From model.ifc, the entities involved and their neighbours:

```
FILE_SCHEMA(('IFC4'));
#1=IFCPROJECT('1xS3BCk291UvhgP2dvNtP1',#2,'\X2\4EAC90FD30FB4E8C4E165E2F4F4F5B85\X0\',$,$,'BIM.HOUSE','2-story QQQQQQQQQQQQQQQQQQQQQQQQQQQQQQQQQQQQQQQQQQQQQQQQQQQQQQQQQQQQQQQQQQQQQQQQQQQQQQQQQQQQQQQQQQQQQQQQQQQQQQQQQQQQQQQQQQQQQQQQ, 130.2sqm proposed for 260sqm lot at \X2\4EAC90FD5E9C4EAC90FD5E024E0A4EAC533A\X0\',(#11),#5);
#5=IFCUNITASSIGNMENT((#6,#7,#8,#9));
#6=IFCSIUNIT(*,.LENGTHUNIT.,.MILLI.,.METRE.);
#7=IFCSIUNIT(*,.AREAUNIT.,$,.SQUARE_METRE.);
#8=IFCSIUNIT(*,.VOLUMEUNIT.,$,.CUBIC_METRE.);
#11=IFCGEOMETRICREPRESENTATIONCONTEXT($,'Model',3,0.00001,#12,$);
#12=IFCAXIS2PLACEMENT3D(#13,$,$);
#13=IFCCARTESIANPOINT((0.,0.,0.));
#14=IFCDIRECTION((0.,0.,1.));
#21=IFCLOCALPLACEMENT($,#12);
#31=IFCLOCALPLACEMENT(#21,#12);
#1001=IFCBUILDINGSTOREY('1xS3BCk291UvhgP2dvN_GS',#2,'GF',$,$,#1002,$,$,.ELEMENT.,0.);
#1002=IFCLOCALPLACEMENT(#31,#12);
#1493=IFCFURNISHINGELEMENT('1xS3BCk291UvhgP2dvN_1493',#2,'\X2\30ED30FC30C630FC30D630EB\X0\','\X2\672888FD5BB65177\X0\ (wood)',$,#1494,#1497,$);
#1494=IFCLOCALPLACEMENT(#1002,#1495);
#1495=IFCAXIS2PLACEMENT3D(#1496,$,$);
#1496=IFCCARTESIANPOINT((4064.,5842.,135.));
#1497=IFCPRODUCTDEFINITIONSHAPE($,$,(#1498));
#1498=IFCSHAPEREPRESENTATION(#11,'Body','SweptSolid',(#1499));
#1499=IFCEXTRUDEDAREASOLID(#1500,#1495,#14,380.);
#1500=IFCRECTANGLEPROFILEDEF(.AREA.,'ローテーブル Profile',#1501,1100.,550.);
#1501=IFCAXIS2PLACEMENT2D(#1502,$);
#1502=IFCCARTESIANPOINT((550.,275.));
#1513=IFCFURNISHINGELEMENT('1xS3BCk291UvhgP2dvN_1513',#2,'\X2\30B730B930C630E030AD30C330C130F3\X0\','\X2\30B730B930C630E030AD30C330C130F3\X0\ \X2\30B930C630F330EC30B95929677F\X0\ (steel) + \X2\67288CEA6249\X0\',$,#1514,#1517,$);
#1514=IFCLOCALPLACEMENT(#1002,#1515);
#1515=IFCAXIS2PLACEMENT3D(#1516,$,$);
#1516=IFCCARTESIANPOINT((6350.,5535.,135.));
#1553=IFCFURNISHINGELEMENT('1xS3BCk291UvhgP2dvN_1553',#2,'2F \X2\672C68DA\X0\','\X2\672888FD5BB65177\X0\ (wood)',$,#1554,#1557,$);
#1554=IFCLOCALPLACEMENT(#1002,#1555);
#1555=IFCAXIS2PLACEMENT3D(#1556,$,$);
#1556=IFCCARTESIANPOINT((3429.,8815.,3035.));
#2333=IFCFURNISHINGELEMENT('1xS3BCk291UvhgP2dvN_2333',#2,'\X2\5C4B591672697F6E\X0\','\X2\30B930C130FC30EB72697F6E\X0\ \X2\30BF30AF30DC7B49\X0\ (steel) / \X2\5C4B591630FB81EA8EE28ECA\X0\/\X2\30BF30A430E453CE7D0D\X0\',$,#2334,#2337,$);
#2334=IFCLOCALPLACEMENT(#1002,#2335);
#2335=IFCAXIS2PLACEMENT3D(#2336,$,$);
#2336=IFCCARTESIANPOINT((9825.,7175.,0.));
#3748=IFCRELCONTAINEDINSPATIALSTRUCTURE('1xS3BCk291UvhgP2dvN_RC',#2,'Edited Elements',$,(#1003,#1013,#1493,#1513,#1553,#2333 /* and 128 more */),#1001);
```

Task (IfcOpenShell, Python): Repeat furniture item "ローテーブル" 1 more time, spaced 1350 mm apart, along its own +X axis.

```python
import ifcopenshell
import ifcopenshell.api.geometry
import ifcopenshell.api.root
import ifcopenshell.util.element
import ifcopenshell.util.placement
import ifcopenshell.util.unit

model = ifcopenshell.open("model.ifc")
unit_scale = ifcopenshell.util.unit.calculate_unit_scale(model)


def reuse_history(source, copy):
    """copy_class also copies each property set's owner history, people and application; keep the originals."""
    for rel in copy.IsDefinedBy:
        if rel.is_a("IfcRelDefinesByProperties") and (history := rel.RelatingPropertyDefinition.OwnerHistory):
            rel.RelatingPropertyDefinition.OwnerHistory = source.OwnerHistory
            ifcopenshell.util.element.remove_deep2(model, history)


source = model.by_guid("1xS3BCk291UvhgP2dvN_1493")
base = ifcopenshell.util.placement.get_local_placement(source.ObjectPlacement)
step = base[:3, 0] * 1.35 / unit_scale

for i in range(1, 2):
    copy = ifcopenshell.api.root.copy_class(model, product=source)
    copy.Representation = ifcopenshell.util.element.copy_deep(
        model, source.Representation, exclude=["IfcGeometricRepresentationContext", "IfcRepresentationMap"]
    )
    reuse_history(source, copy)
    matrix = base.copy()
    matrix[:3, 3] += i * step
    print("added at", matrix[:3, 3].round(3) + 0.0)
    ifcopenshell.api.geometry.edit_object_placement(model, product=copy, matrix=matrix, is_si=False)

model.write("model_edited.ifc")
```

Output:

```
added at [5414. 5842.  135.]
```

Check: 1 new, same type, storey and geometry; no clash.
